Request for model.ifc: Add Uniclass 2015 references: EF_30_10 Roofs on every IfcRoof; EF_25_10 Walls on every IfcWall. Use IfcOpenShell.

First a look at what the model holds.

```python
import ifcopenshell

model = ifcopenshell.open("model.ifc")
print(model.schema)
print("classifications:", [c.Name for c in model.by_type("IfcClassification")])
for ifc_class in ("IfcDoor", "IfcRoof", "IfcStair", "IfcWall", "IfcWindow"):
    print(ifc_class, len(model.by_type(ifc_class)))
```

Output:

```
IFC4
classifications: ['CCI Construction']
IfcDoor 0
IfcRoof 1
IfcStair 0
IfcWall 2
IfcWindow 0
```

```python
import ifcopenshell
import ifcopenshell.api.classification

model = ifcopenshell.open("model.ifc")

system = ifcopenshell.api.classification.add_classification(model, classification="Uniclass 2015")

codes = {
    "IfcRoof": ("EF_30_10", "Roofs"),
    "IfcWall": ("EF_25_10", "Walls"),
}
for ifc_class, (code, name) in codes.items():
    products = model.by_type(ifc_class)
    ifcopenshell.api.classification.add_reference(
        model, products=products, classification=system, identification=code, name=name
    )
    print(code, len(products))

model.write("model_rev.ifc")
```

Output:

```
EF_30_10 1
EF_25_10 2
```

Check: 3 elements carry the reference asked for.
